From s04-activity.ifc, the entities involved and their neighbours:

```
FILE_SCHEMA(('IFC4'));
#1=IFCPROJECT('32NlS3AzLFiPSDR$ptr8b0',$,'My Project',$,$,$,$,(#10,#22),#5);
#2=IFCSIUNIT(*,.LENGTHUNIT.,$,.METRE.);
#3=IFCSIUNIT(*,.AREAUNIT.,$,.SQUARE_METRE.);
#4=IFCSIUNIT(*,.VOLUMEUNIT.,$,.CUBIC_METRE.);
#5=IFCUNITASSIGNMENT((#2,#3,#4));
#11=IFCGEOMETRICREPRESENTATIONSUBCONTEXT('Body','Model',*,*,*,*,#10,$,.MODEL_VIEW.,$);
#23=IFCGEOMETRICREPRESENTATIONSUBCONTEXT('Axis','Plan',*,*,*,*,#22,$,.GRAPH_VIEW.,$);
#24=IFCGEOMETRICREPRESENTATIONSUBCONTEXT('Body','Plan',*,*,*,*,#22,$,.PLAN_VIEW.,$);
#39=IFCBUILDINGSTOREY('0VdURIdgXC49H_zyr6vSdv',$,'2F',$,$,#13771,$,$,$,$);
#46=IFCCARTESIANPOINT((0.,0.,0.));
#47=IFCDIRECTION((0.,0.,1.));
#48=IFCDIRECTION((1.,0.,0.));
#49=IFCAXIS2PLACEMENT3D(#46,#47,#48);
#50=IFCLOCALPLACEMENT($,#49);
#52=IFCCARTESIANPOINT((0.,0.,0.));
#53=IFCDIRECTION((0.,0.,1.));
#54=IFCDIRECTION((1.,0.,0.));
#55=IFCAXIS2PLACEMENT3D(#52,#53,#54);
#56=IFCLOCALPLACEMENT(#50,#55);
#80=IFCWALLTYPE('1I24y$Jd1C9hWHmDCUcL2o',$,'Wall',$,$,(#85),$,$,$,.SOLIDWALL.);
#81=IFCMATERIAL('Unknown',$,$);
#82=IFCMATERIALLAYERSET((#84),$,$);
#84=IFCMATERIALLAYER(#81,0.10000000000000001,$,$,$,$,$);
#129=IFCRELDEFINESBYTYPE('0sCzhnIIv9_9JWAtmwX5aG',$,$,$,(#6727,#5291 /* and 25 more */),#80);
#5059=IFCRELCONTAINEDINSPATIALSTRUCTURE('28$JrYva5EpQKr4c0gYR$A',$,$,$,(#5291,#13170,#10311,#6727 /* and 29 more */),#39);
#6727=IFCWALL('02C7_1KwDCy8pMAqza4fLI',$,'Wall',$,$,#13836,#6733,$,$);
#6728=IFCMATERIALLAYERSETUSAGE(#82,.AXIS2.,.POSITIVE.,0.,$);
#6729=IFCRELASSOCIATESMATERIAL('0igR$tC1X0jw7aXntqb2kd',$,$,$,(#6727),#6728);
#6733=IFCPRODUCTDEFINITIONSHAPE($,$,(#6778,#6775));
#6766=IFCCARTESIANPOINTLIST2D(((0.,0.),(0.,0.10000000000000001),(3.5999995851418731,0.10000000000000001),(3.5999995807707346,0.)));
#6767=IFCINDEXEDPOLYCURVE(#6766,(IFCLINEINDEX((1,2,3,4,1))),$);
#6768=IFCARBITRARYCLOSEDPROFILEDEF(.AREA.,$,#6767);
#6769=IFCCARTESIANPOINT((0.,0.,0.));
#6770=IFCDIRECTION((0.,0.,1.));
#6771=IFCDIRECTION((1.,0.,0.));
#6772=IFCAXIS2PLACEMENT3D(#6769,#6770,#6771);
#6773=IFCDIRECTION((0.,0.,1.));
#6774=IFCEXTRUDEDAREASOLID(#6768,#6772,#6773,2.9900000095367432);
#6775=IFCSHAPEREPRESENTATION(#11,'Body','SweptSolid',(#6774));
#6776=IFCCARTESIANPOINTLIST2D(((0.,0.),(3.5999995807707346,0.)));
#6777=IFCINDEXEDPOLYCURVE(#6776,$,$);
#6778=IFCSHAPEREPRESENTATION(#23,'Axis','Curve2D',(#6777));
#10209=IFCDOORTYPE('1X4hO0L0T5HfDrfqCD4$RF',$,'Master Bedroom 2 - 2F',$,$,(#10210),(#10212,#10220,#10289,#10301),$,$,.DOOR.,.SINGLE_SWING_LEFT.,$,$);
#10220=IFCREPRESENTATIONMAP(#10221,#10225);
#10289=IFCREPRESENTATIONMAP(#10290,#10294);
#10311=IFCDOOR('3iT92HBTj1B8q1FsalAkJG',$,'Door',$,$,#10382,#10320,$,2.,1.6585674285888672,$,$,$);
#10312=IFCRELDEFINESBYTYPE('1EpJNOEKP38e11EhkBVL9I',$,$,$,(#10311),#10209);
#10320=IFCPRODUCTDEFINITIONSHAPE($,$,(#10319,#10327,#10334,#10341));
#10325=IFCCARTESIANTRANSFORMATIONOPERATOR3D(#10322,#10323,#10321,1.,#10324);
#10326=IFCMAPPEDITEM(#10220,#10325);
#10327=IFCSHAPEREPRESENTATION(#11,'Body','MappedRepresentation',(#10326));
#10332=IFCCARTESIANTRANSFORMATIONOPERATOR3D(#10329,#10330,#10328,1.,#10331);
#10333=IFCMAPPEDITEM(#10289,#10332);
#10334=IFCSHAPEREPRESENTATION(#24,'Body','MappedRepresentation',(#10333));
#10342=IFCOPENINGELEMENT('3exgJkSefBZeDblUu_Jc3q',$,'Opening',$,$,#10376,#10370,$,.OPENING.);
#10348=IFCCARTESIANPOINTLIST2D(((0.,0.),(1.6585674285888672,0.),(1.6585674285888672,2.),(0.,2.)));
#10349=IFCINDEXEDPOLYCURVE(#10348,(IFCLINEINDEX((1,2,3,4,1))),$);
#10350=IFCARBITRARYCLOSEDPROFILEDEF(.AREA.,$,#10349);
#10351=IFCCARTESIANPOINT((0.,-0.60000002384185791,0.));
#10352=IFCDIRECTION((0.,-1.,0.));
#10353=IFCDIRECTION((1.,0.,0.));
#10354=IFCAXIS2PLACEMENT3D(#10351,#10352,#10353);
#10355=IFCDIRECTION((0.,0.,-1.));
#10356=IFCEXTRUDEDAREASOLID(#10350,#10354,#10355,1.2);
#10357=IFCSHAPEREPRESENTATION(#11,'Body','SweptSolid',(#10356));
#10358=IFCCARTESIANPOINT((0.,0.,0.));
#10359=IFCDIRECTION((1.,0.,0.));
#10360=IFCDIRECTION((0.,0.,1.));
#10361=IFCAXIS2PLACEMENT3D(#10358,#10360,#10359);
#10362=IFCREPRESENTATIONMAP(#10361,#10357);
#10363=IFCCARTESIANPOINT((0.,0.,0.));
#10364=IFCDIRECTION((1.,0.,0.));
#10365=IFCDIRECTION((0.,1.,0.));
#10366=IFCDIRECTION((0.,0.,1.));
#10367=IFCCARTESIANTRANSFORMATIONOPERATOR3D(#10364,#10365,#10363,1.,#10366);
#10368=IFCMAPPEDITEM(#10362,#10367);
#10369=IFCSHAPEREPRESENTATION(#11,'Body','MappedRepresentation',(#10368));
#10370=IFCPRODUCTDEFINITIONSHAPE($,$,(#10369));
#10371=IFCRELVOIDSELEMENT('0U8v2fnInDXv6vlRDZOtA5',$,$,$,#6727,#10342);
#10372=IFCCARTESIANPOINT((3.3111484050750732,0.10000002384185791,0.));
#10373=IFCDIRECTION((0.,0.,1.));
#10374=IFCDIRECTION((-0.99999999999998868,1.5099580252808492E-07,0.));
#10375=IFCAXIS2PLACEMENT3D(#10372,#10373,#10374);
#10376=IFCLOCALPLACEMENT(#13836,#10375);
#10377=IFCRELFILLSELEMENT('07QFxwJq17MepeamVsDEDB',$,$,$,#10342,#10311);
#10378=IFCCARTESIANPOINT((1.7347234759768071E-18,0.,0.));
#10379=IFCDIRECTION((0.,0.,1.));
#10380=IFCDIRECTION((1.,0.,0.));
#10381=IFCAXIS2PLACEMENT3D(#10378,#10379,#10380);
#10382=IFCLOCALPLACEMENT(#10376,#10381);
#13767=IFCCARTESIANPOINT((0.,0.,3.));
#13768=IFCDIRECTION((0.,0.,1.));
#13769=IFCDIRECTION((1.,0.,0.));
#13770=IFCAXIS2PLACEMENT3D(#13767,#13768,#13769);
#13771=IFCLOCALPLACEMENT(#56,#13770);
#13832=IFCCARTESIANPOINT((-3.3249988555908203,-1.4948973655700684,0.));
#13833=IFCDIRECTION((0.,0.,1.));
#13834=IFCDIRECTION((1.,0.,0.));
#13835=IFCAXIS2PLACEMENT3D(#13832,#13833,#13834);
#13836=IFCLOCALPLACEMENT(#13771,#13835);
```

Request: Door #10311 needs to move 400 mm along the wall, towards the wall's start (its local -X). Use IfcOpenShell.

```python
import ifcopenshell
import ifcopenshell.api.geometry
import ifcopenshell.util.placement
import ifcopenshell.util.unit

model = ifcopenshell.open("s04-activity.ifc")
unit_scale = ifcopenshell.util.unit.calculate_unit_scale(model)

door = model.by_id(10311)
opening = door.FillsVoids[0].RelatingOpeningElement
wall = opening.VoidsElements[0].RelatingBuildingElement

wall_matrix = ifcopenshell.util.placement.get_local_placement(wall.ObjectPlacement)
shift = wall_matrix[:3, 0] * -0.4 / unit_scale
before = ifcopenshell.util.placement.get_local_placement(door.ObjectPlacement)[:3, 3].copy()

# The door is placed relative to its opening, so it follows when the opening moves.
matrix = ifcopenshell.util.placement.get_local_placement(opening.ObjectPlacement)
matrix[:3, 3] += shift
ifcopenshell.api.geometry.edit_object_placement(
    model, product=opening, matrix=matrix, is_si=False, should_transform_children=True
)

after = ifcopenshell.util.placement.get_local_placement(door.ObjectPlacement)[:3, 3]
print("door moved by", (after - before).round(3) + 0.0)

model.write("s04-activity-out.ifc")
```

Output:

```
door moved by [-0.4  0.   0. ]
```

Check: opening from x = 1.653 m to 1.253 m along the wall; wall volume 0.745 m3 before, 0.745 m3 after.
